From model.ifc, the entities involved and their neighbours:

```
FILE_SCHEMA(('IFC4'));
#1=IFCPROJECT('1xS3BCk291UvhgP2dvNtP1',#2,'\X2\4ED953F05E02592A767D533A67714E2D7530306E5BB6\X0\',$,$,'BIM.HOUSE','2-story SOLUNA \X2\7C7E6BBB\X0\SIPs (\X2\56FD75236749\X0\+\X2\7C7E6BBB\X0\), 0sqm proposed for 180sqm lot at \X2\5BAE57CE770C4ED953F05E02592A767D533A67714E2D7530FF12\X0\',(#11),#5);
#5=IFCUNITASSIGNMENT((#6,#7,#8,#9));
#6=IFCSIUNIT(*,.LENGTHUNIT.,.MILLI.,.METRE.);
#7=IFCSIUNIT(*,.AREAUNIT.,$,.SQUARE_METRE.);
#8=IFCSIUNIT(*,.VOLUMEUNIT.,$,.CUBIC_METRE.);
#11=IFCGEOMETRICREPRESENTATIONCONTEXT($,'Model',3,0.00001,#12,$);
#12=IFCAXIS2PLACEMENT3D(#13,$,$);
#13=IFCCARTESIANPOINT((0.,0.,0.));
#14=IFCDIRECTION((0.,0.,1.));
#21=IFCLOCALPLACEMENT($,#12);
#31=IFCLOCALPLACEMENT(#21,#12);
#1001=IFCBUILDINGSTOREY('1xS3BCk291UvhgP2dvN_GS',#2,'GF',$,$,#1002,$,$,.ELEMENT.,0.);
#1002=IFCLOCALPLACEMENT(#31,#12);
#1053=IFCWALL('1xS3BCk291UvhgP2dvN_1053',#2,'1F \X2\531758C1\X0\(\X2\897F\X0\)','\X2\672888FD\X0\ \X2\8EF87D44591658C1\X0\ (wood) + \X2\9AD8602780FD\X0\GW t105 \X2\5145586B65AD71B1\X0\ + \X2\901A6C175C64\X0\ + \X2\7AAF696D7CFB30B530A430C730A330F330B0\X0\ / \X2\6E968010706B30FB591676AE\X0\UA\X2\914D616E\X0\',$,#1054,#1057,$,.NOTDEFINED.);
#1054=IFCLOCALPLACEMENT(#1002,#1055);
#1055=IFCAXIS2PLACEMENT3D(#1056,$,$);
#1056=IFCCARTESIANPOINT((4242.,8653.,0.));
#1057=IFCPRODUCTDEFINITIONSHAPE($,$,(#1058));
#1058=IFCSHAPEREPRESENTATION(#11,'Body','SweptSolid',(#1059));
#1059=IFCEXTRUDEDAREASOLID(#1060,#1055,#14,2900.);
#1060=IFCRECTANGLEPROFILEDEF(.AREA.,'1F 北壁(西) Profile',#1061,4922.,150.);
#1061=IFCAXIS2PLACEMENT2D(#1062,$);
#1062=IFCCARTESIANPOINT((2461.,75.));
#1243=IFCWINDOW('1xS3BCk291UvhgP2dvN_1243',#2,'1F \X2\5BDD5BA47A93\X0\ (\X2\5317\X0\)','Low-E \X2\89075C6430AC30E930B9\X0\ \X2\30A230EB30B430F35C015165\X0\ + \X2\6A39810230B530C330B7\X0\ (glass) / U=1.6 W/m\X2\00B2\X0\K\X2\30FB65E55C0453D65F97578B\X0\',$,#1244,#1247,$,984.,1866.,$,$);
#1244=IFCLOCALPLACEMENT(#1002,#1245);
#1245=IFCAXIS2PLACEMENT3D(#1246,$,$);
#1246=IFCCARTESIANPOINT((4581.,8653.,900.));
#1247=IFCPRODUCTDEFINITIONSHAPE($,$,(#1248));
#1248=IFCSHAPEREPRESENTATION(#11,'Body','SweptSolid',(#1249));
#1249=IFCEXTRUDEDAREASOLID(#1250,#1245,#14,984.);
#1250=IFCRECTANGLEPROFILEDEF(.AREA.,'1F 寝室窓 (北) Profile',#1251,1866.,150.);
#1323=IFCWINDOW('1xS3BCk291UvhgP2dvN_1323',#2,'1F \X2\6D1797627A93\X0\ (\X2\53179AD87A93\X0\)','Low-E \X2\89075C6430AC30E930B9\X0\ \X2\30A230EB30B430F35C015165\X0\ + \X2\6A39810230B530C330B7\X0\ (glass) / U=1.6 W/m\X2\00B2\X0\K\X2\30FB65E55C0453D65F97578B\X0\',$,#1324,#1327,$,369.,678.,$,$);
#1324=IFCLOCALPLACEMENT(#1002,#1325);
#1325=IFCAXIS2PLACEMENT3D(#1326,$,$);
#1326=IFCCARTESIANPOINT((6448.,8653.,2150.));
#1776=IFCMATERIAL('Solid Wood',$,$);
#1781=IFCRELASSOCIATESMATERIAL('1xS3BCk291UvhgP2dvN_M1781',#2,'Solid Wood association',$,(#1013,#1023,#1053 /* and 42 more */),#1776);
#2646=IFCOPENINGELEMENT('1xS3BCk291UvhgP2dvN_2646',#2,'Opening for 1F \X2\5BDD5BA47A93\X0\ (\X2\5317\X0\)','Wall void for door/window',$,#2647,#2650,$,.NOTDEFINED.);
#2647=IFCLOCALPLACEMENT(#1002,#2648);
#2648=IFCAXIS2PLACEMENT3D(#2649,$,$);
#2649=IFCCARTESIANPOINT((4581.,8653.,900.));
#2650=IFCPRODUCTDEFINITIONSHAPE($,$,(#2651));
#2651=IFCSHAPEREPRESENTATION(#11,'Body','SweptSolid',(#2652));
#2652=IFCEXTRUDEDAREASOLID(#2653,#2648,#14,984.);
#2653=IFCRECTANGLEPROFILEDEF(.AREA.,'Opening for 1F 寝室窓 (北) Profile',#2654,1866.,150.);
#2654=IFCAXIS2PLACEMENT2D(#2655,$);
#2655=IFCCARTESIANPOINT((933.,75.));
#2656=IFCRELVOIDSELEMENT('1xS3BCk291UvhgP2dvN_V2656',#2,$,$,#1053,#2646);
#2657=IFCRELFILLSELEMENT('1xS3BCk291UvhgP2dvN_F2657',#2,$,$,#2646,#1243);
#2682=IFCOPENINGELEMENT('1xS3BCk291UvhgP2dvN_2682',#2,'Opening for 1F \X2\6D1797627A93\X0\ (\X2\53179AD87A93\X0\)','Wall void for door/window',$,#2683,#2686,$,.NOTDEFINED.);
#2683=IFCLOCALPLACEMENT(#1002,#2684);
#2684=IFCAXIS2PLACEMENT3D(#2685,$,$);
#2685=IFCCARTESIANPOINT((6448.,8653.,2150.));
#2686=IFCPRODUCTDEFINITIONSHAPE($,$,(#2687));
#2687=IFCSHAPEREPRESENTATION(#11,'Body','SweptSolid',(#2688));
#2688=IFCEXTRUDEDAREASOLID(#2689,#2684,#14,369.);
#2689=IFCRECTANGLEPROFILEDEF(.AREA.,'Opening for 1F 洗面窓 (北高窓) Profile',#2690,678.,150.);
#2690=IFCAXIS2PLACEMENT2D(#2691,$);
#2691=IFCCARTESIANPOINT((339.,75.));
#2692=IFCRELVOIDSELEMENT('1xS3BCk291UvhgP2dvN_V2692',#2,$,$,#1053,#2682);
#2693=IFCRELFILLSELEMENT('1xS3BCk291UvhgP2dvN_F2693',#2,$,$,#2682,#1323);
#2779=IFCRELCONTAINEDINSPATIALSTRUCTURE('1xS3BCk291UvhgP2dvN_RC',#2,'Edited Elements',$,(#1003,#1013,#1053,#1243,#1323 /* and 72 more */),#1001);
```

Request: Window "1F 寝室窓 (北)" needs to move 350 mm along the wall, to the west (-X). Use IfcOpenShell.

```python
import ifcopenshell
import ifcopenshell.api.geometry
import ifcopenshell.util.placement

model = ifcopenshell.open("model.ifc")

window = model.by_guid("1xS3BCk291UvhgP2dvN_1243")
opening = window.FillsVoids[0].RelatingOpeningElement
wall = opening.VoidsElements[0].RelatingBuildingElement

wall_matrix = ifcopenshell.util.placement.get_local_placement(wall.ObjectPlacement)
shift = wall_matrix[:3, 0] * -350.0
before = ifcopenshell.util.placement.get_local_placement(window.ObjectPlacement)[:3, 3].copy()

# The window is not placed relative to its opening, so move both.
for product in (opening, window):
    matrix = ifcopenshell.util.placement.get_local_placement(product.ObjectPlacement)
    matrix[:3, 3] += shift
    ifcopenshell.api.geometry.edit_object_placement(model, product=product, matrix=matrix, is_si=False)

after = ifcopenshell.util.placement.get_local_placement(window.ObjectPlacement)[:3, 3]
print("window moved by", (after - before).round(3) + 0.0)

model.write("model_edited.ifc")
```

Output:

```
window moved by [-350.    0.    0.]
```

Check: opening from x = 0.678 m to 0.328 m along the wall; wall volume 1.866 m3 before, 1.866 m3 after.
